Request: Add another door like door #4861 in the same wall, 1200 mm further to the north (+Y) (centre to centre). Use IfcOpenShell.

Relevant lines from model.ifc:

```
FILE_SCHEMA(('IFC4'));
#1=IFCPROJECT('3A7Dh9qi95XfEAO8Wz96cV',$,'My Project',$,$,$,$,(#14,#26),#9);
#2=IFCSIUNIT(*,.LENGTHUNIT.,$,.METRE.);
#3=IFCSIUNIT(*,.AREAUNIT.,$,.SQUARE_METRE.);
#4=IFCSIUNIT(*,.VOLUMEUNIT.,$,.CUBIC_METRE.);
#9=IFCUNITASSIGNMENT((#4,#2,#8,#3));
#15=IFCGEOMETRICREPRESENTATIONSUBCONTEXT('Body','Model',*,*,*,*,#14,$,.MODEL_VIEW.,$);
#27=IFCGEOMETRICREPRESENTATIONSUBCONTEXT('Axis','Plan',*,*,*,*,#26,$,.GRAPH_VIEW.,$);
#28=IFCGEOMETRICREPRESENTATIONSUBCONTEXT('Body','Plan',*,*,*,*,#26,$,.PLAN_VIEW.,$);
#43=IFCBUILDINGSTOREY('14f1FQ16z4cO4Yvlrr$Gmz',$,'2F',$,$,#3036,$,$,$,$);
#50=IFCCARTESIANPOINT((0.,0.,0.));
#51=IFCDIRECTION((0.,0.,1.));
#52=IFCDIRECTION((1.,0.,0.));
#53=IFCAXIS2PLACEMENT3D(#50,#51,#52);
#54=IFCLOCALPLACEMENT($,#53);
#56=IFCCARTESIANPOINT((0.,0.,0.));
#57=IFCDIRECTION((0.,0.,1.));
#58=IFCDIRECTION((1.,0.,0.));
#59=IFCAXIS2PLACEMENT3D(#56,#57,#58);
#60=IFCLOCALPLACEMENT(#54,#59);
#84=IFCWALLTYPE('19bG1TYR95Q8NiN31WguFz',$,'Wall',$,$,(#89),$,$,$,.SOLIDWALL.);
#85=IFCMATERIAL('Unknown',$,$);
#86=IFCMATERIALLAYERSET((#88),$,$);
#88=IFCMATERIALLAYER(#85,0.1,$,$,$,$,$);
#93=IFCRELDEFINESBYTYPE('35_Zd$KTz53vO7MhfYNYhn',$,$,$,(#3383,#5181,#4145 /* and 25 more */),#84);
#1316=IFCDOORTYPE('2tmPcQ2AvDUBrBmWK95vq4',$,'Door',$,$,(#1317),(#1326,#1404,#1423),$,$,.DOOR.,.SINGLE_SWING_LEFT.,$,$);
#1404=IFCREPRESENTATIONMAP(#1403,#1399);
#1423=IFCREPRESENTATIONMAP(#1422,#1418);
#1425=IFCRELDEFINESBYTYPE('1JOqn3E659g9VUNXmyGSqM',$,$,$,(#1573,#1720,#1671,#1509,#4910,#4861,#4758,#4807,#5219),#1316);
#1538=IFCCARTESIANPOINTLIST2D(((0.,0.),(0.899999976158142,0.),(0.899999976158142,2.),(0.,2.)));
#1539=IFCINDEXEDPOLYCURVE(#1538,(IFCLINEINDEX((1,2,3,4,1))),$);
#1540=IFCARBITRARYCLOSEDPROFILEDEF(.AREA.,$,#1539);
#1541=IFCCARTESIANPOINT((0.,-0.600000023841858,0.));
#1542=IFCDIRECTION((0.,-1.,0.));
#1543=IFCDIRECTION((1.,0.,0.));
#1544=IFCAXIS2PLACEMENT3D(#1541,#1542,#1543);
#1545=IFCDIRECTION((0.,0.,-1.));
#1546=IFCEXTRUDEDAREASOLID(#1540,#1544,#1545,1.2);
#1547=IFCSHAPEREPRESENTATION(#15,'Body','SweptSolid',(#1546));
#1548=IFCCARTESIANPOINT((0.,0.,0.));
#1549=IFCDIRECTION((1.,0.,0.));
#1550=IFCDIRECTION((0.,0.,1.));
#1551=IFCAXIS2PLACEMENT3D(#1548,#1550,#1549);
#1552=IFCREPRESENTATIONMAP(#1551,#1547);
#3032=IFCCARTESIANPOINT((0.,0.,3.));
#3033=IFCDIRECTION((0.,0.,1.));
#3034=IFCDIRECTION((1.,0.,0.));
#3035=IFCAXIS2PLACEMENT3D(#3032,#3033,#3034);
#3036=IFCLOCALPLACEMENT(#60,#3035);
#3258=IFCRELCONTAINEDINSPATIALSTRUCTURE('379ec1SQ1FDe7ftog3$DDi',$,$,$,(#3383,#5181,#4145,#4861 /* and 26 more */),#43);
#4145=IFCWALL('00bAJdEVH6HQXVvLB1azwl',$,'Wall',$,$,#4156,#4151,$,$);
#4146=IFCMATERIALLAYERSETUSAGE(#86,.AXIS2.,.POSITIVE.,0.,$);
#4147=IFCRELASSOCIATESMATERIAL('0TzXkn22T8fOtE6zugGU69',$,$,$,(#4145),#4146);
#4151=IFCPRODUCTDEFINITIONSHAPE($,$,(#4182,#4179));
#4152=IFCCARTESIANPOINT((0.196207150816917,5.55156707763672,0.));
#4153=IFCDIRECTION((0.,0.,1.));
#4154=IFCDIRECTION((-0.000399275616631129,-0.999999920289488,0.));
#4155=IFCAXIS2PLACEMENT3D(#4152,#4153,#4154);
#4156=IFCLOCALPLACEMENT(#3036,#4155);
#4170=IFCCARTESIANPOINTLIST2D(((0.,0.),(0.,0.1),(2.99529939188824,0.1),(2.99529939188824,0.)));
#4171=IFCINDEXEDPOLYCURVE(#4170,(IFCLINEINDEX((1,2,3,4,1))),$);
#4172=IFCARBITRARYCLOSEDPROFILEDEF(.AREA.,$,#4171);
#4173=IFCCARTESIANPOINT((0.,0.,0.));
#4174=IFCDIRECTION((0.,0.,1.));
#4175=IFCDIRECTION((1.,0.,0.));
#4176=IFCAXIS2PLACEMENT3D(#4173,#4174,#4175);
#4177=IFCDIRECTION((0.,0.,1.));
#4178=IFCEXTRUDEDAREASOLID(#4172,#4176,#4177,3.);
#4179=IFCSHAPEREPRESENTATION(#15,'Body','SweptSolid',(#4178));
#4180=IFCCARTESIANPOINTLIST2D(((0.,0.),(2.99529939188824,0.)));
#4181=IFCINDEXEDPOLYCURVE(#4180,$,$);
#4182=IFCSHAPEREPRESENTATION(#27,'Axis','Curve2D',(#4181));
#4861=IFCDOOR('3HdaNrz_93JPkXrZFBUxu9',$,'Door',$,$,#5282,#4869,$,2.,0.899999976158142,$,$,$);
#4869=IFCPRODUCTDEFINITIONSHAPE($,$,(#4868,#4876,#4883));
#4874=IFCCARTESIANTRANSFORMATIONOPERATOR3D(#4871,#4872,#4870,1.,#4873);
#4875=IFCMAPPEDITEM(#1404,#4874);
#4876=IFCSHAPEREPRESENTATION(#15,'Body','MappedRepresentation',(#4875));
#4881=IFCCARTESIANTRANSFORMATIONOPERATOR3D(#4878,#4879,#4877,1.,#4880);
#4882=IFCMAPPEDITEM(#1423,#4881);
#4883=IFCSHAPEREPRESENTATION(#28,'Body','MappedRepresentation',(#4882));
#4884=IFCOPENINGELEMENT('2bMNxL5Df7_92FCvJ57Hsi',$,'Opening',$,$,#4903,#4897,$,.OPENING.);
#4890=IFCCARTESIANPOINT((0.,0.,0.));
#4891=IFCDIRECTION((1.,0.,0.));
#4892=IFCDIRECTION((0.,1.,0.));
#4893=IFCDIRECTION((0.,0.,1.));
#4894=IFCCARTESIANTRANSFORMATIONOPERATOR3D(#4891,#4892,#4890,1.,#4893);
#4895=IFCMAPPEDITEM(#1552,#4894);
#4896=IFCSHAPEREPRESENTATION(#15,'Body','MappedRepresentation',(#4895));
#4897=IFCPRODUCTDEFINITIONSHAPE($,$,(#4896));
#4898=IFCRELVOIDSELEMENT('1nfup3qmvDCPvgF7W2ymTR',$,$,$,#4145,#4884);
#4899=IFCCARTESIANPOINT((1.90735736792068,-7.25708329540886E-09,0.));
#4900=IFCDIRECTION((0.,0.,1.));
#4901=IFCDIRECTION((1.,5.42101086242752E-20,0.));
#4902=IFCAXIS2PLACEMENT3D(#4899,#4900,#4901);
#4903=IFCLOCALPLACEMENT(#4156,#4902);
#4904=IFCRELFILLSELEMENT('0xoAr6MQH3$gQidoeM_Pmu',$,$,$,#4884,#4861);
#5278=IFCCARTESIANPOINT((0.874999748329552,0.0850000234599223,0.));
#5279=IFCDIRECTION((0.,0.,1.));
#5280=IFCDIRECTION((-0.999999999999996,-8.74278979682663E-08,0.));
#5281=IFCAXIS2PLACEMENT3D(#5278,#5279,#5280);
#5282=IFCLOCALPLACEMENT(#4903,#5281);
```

```python
import ifcopenshell
import ifcopenshell.api.feature
import ifcopenshell.api.geometry
import ifcopenshell.api.root
import ifcopenshell.geom
import ifcopenshell.util.element
import ifcopenshell.util.placement
import ifcopenshell.util.shape
import ifcopenshell.util.unit

model = ifcopenshell.open("model.ifc")
unit_scale = ifcopenshell.util.unit.calculate_unit_scale(model)
settings = ifcopenshell.geom.settings()


def volume(element):
    """Net volume in cubic metres, openings subtracted."""
    shape = ifcopenshell.geom.create_shape(settings, element)
    return ifcopenshell.util.shape.get_volume(shape.geometry)


door = model.by_guid("3HdaNrz_93JPkXrZFBUxu9")
opening = door.FillsVoids[0].RelatingOpeningElement
wall = opening.VoidsElements[0].RelatingBuildingElement
before = volume(wall)
shift = ifcopenshell.util.placement.get_local_placement(wall.ObjectPlacement)[:3, 0] * -1.2 / unit_scale

# copy_class copies the void relationship, type, container and properties, but no geometry.
new_opening = ifcopenshell.api.root.copy_class(model, product=opening)
new_opening.Representation = ifcopenshell.util.element.copy_deep(
    model, opening.Representation, exclude=["IfcGeometricRepresentationContext", "IfcRepresentationMap"]
)
new_door = ifcopenshell.api.root.copy_class(model, product=door)
new_door.Representation = ifcopenshell.util.element.copy_deep(
    model, door.Representation, exclude=["IfcGeometricRepresentationContext", "IfcRepresentationMap"]
)
ifcopenshell.api.feature.add_filling(model, opening=new_opening, element=new_door)

for old, new in ((opening, new_opening), (door, new_door)):
    matrix = ifcopenshell.util.placement.get_local_placement(old.ObjectPlacement)
    matrix[:3, 3] += shift
    ifcopenshell.api.geometry.edit_object_placement(model, product=new, matrix=matrix, is_si=False)

after = volume(wall)

print(f"wall volume {before:.3f} -> {after:.3f} m3")

model.write("model-out.ifc")
```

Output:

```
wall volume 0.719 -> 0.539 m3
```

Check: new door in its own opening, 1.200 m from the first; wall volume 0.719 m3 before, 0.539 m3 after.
